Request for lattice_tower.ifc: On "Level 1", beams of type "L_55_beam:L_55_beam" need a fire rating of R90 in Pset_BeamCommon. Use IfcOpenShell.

First a look at what the model holds.

```python
import ifcopenshell
import ifcopenshell.util.element

model = ifcopenshell.open("lattice_tower.ifc")
print(model.schema)
storey = next(s for s in model.by_type("IfcBuildingStorey") if s.Name == "Level 1")
beams = [e for e in ifcopenshell.util.element.get_decomposition(storey) if e.is_a("IfcBeam")]
seen = {}
for e in beams:
    element_type = ifcopenshell.util.element.get_type(e)
    key = (element_type.Name if element_type != e and element_type else None, ifcopenshell.util.element.get_pset(e, "Pset_BeamCommon", "FireRating"))
    seen[key] = seen.get(key, 0) + 1
for (name, value), count in sorted(seen.items(), key=str):
    print(count, "x", name, "|", value)
```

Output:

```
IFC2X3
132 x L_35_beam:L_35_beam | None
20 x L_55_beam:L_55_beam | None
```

```python
import ifcopenshell
import ifcopenshell.api.pset
import ifcopenshell.util.element

model = ifcopenshell.open("lattice_tower.ifc")

storey = next(s for s in model.by_type("IfcBuildingStorey") if s.Name == "Level 1")
beams = [e for e in ifcopenshell.util.element.get_decomposition(storey) if e.is_a("IfcBeam")]

count = 0
for e in beams:
    element_type = ifcopenshell.util.element.get_type(e)
    if element_type in (None, e) or element_type.Name != "L_55_beam:L_55_beam":
        continue
    # add_pset returns the element's existing set when there is one.
    pset = ifcopenshell.api.pset.add_pset(model, product=e, name="Pset_BeamCommon")
    ifcopenshell.api.pset.edit_pset(model, pset=pset, properties={"FireRating": "R90"})
    count += 1

print(count, "beams updated")

model.write("lattice_tower_edited.ifc")
```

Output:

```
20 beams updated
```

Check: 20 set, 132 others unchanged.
